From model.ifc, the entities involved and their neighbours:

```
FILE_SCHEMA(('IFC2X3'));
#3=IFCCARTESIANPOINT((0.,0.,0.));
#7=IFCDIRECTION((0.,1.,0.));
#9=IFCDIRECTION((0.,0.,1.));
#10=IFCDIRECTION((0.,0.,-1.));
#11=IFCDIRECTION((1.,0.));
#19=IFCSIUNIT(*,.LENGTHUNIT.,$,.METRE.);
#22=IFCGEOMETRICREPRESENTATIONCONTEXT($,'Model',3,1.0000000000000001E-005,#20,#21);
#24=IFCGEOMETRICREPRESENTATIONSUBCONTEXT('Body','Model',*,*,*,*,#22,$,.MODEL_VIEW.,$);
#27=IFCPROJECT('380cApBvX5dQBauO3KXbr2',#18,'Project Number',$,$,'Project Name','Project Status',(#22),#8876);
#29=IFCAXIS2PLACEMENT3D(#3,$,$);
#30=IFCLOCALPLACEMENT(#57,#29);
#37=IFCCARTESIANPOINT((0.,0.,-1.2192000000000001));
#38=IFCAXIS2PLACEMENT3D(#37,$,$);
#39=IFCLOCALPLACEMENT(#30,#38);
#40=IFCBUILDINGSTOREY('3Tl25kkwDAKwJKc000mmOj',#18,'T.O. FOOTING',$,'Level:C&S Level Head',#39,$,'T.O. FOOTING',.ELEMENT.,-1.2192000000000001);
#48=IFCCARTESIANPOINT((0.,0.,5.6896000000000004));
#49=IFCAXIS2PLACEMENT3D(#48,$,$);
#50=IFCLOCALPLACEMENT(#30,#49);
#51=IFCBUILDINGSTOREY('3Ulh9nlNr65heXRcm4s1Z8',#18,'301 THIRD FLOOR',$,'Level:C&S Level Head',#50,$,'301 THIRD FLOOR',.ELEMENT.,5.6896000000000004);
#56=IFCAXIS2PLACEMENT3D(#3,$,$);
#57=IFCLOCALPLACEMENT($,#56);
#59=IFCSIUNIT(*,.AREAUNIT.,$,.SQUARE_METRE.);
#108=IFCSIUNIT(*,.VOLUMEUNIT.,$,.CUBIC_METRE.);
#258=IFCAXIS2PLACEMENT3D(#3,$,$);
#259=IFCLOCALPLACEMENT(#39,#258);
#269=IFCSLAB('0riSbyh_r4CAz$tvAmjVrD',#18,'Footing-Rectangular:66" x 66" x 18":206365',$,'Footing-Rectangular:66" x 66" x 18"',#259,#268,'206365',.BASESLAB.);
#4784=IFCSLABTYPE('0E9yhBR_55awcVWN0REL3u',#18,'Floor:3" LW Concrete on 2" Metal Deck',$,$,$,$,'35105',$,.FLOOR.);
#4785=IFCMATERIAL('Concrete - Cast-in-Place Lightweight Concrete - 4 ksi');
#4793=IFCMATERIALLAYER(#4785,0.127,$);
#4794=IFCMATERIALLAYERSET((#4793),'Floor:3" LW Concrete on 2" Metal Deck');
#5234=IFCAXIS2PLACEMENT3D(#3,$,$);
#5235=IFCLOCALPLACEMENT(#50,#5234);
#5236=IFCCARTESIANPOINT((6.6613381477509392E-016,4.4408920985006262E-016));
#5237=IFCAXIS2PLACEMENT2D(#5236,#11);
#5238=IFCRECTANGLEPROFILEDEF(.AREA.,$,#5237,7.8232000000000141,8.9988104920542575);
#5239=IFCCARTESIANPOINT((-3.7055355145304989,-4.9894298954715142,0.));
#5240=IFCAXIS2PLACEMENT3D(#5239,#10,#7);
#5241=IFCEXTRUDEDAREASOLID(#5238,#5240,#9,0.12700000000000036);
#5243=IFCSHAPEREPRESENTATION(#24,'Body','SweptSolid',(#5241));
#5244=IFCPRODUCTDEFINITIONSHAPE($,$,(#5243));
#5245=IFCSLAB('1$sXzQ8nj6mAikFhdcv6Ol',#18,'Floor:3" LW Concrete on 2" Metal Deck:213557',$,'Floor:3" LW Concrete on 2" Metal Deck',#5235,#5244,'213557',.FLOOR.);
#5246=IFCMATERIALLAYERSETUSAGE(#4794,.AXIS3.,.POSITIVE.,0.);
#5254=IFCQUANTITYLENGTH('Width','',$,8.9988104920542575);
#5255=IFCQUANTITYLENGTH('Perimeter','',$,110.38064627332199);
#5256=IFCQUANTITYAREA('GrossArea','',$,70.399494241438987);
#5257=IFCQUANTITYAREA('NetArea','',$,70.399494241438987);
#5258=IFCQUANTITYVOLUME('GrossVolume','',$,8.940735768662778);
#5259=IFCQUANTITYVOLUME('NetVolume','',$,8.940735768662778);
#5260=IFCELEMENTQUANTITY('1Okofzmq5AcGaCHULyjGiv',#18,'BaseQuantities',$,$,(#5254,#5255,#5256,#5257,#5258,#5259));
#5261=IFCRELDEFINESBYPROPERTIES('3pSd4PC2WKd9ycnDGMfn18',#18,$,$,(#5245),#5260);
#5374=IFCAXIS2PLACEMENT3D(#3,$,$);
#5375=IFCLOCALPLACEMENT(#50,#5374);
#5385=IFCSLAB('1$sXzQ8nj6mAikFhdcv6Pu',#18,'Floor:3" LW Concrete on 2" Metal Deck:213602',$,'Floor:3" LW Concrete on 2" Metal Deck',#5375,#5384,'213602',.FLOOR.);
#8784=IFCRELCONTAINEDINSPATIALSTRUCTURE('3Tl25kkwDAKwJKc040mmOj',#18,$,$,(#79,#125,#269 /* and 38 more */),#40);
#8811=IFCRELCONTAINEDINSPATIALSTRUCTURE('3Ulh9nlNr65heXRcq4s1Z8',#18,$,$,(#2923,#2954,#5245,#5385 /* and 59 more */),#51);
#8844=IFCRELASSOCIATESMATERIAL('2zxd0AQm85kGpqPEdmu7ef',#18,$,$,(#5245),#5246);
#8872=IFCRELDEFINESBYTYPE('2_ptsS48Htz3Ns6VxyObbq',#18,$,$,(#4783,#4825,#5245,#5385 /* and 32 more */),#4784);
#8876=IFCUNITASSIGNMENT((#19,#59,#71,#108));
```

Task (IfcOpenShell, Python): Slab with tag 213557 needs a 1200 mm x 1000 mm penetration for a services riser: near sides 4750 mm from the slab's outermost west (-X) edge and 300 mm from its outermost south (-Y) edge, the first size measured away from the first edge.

```python
import numpy as np
import ifcopenshell
import ifcopenshell.api.feature
import ifcopenshell.api.geometry
import ifcopenshell.api.pset
import ifcopenshell.api.root
import ifcopenshell.geom
import ifcopenshell.util.element
import ifcopenshell.util.placement
import ifcopenshell.util.representation
import ifcopenshell.util.shape
import ifcopenshell.util.unit

model = ifcopenshell.open("model.ifc")
unit_scale = ifcopenshell.util.unit.calculate_unit_scale(model)
area_scale = ifcopenshell.util.unit.calculate_unit_scale(model, "AREAUNIT")
volume_scale = ifcopenshell.util.unit.calculate_unit_scale(model, "VOLUMEUNIT")
settings = ifcopenshell.geom.settings()


def volume(element):
    """Net volume in cubic metres, openings subtracted."""
    shape = ifcopenshell.geom.create_shape(settings, element)
    return ifcopenshell.util.shape.get_volume(shape.geometry)


slab = model.by_guid("1$sXzQ8nj6mAikFhdcv6Ol")
before = volume(slab)

# Extent in the slab's own axes, in metres. The edges named are its -X and -Y sides.
slab_shape = ifcopenshell.geom.create_shape(settings, slab)
vertices = ifcopenshell.util.shape.get_vertices(slab_shape.geometry)
x_min, y_min, bottom = vertices.min(axis=0)
top = vertices[:, 2].max()

opening = ifcopenshell.api.root.create_entity(model, ifc_class="IfcOpeningElement", name="Services riser opening")
context = ifcopenshell.util.representation.get_context(model, "Model", "Body", "MODEL_VIEW")
width, depth = 1.2, 1
outline = [(0.0, 0.0), (width, 0.0), (width, depth), (0.0, depth), (0.0, 0.0)]
# Overshoot both faces by 50 mm so the cut is clean.
shape = ifcopenshell.api.geometry.add_slab_representation(
    model, context=context, depth=top - bottom + 0.1, polyline=outline
)
ifcopenshell.api.geometry.assign_representation(model, product=opening, representation=shape)

matrix = ifcopenshell.util.placement.get_local_placement(slab.ObjectPlacement)
matrix[:, 3] = matrix @ np.append(np.array([x_min + 4.75, y_min + 0.3, bottom - 0.05]) / unit_scale, 1.0)
ifcopenshell.api.geometry.edit_object_placement(model, product=opening, matrix=matrix, is_si=False)
ifcopenshell.api.feature.add_feature(model, feature=opening, element=slab)

after = volume(slab)

# Update the slab's stored quantities.
qto = model.by_id(ifcopenshell.util.element.get_pset(slab, "BaseQuantities", should_inherit=False)["id"])
ifcopenshell.api.pset.edit_qto(model, qto=qto, properties={
    "NetArea": after / (top - bottom) / area_scale,
    "NetVolume": after / volume_scale,
})

print(f"slab volume {before:.3f} -> {after:.3f} m3")

model.write("model-out.ifc")
```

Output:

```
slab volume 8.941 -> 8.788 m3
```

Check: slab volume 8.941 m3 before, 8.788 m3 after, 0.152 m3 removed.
